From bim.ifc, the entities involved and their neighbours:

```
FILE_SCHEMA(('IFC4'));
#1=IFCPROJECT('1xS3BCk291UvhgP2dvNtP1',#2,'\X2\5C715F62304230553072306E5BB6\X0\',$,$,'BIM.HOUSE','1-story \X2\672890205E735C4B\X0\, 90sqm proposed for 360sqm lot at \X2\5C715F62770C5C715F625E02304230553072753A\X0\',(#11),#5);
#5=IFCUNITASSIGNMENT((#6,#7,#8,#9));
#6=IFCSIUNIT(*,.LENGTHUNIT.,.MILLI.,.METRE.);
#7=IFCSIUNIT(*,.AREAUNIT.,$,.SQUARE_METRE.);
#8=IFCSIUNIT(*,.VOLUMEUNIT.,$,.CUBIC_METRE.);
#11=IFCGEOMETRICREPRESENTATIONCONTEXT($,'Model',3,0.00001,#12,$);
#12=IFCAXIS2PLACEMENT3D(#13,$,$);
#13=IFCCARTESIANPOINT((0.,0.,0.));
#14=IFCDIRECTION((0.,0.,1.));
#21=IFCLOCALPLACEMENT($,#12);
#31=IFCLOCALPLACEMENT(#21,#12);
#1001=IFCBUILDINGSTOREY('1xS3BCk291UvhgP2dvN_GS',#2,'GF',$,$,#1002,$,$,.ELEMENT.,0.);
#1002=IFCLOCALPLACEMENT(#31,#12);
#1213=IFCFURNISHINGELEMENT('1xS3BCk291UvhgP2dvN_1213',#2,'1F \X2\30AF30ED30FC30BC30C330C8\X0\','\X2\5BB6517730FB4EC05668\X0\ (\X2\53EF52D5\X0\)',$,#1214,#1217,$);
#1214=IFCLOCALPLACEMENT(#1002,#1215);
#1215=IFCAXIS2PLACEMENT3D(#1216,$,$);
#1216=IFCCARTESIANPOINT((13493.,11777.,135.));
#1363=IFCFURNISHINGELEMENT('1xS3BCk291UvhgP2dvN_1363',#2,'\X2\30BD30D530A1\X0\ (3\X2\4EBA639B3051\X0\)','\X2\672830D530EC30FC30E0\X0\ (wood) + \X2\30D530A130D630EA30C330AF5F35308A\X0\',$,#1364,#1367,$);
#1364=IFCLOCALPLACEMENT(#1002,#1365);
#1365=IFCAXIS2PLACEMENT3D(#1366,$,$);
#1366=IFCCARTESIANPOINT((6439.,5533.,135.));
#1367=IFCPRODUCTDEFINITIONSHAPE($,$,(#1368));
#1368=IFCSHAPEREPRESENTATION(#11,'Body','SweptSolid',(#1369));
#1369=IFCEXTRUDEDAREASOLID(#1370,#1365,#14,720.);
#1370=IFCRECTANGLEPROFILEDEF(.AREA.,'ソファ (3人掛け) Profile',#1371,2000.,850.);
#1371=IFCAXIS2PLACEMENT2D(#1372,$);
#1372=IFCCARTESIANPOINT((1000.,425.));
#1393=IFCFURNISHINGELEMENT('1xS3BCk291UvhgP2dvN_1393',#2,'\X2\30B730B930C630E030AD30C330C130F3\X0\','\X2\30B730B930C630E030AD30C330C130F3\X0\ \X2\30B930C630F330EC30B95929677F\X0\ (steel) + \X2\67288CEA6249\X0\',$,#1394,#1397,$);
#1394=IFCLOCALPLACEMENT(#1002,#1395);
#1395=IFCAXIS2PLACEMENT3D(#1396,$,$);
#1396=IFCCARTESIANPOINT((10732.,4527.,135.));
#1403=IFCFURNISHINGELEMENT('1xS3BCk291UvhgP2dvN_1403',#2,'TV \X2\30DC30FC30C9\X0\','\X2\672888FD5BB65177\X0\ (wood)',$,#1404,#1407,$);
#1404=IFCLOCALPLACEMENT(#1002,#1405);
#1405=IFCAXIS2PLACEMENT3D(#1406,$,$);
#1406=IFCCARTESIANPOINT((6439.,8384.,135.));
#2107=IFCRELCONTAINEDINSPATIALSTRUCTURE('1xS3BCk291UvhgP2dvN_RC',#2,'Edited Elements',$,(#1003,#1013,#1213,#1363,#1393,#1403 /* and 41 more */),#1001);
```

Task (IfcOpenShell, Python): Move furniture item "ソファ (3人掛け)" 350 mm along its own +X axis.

```python
import ifcopenshell
import ifcopenshell.api.geometry
import ifcopenshell.util.placement

model = ifcopenshell.open("bim.ifc")

item = model.by_guid("1xS3BCk291UvhgP2dvN_1363")
matrix = ifcopenshell.util.placement.get_local_placement(item.ObjectPlacement)
matrix[:3, 3] += matrix[:3, 0] * 350.0
ifcopenshell.api.geometry.edit_object_placement(model, product=item, matrix=matrix, is_si=False)

print(ifcopenshell.util.placement.get_local_placement(item.ObjectPlacement).round(3) + 0.0)

model.write("bim_rev.ifc")
```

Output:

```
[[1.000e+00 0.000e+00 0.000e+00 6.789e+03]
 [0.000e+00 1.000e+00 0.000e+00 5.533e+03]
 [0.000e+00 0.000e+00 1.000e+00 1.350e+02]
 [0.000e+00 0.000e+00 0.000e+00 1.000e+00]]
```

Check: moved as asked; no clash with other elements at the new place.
